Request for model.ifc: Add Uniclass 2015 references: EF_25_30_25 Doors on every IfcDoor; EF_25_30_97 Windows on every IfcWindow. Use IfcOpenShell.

First a look at what the model holds.

```python
import ifcopenshell

model = ifcopenshell.open("model.ifc")
print(model.schema)
print("classifications:", [c.Name for c in model.by_type("IfcClassification")])
for ifc_class in ("IfcDoor", "IfcRoof", "IfcStair", "IfcWall", "IfcWindow"):
    print(ifc_class, len(model.by_type(ifc_class)))
```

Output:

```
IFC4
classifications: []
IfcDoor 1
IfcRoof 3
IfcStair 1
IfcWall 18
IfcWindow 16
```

```python
import ifcopenshell
import ifcopenshell.api.classification

model = ifcopenshell.open("model.ifc")

system = ifcopenshell.api.classification.add_classification(model, classification="Uniclass 2015")

codes = {
    "IfcDoor": ("EF_25_30_25", "Doors"),
    "IfcWindow": ("EF_25_30_97", "Windows"),
}
for ifc_class, (code, name) in codes.items():
    products = model.by_type(ifc_class)
    ifcopenshell.api.classification.add_reference(
        model, products=products, classification=system, identification=code, name=name
    )
    print(code, len(products))

model.write("model_rev.ifc")
```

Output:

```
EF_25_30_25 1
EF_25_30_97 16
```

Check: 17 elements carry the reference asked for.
